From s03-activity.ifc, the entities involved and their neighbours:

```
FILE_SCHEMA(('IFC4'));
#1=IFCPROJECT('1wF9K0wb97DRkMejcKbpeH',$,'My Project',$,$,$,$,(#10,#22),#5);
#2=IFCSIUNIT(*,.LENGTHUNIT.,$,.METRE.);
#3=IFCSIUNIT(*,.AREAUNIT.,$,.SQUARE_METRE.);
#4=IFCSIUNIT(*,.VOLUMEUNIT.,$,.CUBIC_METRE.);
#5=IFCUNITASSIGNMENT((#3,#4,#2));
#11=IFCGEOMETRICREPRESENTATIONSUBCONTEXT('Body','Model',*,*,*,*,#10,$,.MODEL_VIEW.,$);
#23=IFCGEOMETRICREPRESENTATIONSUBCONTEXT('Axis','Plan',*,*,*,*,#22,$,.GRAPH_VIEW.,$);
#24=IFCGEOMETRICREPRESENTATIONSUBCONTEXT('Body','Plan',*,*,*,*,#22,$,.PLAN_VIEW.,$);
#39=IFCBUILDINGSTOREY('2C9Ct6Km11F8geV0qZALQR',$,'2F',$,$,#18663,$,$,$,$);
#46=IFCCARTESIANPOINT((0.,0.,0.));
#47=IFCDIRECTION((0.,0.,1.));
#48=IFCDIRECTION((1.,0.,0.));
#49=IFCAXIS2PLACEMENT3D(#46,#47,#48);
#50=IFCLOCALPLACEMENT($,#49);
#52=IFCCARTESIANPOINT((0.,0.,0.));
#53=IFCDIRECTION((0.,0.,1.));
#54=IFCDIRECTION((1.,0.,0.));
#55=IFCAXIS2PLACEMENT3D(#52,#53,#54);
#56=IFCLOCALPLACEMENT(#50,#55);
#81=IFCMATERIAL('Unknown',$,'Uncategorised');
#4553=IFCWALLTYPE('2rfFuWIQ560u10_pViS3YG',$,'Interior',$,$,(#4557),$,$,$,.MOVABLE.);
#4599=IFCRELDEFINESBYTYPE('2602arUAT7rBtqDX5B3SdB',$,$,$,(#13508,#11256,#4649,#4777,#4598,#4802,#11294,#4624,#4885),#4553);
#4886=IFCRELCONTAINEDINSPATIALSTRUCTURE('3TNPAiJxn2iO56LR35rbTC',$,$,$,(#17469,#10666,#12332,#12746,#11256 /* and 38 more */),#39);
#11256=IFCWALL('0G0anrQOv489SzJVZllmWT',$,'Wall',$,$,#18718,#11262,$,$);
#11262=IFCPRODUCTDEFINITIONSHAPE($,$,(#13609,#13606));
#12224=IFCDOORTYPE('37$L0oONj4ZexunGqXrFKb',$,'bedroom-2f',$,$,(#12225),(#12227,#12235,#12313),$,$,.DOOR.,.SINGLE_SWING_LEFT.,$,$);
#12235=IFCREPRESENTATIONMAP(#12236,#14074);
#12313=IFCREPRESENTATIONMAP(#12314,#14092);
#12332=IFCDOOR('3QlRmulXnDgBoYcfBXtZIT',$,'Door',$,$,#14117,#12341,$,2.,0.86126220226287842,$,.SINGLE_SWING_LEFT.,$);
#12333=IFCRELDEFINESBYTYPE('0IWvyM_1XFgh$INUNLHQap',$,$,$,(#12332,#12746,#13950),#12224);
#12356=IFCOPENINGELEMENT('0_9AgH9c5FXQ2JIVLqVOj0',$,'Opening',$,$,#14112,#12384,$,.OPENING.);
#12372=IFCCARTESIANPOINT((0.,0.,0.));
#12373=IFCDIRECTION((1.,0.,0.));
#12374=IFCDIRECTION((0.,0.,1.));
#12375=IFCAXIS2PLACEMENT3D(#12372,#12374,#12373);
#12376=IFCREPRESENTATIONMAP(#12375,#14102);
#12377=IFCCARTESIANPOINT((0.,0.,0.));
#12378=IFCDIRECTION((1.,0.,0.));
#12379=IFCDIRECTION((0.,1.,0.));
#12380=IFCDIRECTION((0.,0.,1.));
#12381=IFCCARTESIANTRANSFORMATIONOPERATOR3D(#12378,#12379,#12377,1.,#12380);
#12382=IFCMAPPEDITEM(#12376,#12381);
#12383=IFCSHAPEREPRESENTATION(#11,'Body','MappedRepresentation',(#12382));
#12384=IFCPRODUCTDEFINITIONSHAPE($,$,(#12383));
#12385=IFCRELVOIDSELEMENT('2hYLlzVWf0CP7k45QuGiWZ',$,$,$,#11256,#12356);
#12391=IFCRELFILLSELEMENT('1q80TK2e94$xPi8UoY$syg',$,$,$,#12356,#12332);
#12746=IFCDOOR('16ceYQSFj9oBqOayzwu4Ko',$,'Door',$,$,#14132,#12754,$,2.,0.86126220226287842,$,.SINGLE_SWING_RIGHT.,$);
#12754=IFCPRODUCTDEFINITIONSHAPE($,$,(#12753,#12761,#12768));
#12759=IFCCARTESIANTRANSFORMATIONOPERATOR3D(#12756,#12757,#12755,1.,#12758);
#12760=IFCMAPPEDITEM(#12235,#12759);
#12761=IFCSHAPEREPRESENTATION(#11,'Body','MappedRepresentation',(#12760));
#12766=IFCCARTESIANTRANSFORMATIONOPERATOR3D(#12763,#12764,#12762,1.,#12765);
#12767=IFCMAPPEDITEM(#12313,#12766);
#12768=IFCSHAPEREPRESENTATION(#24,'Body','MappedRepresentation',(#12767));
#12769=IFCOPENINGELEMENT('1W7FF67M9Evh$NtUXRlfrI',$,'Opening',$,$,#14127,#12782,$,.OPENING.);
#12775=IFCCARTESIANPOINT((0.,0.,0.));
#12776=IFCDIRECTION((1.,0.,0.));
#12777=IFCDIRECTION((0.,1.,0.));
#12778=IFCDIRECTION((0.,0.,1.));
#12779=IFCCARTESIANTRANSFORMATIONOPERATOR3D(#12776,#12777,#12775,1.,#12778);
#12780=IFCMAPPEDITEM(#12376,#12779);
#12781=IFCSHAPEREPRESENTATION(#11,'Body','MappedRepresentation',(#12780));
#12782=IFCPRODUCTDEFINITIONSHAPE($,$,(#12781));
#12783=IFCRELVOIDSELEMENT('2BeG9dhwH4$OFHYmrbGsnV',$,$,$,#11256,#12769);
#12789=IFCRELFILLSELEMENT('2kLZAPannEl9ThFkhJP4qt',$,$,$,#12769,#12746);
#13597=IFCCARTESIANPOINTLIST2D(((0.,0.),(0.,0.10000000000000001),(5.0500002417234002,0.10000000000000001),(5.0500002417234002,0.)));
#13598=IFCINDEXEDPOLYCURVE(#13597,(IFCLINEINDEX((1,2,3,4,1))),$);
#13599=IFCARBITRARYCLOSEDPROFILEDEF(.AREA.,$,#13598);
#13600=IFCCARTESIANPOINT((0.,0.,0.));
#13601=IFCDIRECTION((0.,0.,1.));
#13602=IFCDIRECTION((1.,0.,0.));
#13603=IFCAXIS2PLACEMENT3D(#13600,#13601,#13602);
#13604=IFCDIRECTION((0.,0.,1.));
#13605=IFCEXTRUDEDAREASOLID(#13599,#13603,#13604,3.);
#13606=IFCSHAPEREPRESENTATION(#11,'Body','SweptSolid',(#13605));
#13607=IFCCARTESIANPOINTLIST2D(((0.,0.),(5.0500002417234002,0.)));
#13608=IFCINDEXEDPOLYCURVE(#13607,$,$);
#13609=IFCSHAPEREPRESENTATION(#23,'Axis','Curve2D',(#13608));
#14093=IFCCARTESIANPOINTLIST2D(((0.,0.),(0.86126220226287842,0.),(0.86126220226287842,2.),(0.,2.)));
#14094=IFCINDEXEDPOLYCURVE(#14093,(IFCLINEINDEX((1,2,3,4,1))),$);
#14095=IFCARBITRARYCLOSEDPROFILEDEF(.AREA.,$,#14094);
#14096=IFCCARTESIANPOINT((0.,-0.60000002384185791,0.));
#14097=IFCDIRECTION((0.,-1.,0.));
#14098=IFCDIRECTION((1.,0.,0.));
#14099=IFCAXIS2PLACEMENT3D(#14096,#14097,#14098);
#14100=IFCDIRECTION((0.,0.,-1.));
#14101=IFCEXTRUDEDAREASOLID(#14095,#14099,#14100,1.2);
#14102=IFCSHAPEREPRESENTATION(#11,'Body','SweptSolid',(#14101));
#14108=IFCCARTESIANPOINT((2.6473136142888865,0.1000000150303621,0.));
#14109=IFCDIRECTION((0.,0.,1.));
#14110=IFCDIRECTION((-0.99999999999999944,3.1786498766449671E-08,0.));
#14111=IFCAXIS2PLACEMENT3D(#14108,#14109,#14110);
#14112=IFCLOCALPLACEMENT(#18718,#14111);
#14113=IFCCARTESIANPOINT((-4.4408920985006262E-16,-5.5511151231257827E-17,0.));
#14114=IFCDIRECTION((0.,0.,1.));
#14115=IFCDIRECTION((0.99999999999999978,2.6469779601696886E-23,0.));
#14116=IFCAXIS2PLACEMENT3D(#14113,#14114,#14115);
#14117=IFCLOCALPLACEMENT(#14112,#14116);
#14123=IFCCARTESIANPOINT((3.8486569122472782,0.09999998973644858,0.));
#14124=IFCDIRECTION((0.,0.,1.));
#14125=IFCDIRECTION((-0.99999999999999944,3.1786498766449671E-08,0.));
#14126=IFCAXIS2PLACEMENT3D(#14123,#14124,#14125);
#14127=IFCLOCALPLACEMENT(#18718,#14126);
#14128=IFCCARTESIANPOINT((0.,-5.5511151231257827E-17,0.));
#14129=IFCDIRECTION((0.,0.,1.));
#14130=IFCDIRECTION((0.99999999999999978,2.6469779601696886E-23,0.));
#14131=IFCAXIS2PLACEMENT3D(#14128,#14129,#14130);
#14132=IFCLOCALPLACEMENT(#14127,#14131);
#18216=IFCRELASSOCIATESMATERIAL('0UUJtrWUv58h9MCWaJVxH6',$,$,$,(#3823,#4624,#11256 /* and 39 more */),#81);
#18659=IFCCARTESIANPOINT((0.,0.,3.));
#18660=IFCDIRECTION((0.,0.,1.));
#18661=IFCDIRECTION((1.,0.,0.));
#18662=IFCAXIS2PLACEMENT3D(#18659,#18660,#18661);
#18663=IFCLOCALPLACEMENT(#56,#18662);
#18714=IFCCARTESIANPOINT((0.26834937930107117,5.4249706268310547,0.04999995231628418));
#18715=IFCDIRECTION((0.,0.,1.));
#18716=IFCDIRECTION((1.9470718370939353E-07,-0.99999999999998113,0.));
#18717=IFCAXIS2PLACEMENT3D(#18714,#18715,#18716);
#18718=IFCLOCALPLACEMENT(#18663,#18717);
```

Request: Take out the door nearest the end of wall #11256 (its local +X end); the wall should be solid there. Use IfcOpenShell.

```python
import ifcopenshell
import ifcopenshell.api.feature
import ifcopenshell.api.root
import ifcopenshell.geom
import ifcopenshell.util.shape

model = ifcopenshell.open("s03-activity.ifc")
settings = ifcopenshell.geom.settings()


def volume(element):
    """Net volume in cubic metres, openings subtracted."""
    shape = ifcopenshell.geom.create_shape(settings, element)
    return ifcopenshell.util.shape.get_volume(shape.geometry)


door = model.by_guid("16ceYQSFj9oBqOayzwu4Ko")
opening = door.FillsVoids[0].RelatingOpeningElement
wall = opening.VoidsElements[0].RelatingBuildingElement
before = volume(wall)

ifcopenshell.api.root.remove_product(model, product=door)
ifcopenshell.api.feature.remove_feature(model, feature=opening)

after = volume(wall)

print(f"wall volume {before:.3f} -> {after:.3f} m3")

model.write("s03-activity_v2.ifc")
```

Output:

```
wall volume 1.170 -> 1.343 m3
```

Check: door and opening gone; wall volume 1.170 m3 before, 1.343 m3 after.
